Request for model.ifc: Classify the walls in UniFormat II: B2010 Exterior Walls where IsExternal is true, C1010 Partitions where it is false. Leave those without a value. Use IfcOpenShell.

First a look at what the model holds.

```python
import ifcopenshell
import ifcopenshell.util.element

model = ifcopenshell.open("model.ifc")
print(model.schema)
print("classifications:", [c.Name for c in model.by_type("IfcClassification")])
values = [ifcopenshell.util.element.get_pset(e, "Pset_WallCommon", "IsExternal") for e in model.by_type("IfcWall")]
for value in (True, False, None):
    print("IsExternal", value, values.count(value))
```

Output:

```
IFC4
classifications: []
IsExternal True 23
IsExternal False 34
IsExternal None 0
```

```python
import ifcopenshell
import ifcopenshell.api.classification
import ifcopenshell.util.element

model = ifcopenshell.open("model.ifc")

system = ifcopenshell.api.classification.add_classification(model, classification="UniFormat II")

walls = model.by_type("IfcWall")
external = {e: ifcopenshell.util.element.get_pset(e, "Pset_WallCommon", "IsExternal") for e in walls}
for flag, code, name in ((True, "B2010", "Exterior Walls"), (False, "C1010", "Partitions")):
    products = [e for e in walls if external[e] is flag]
    ifcopenshell.api.classification.add_reference(
        model, products=products, classification=system, identification=code, name=name
    )
    print(code, len(products))

model.write("model-out.ifc")
```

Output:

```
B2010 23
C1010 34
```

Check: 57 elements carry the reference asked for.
